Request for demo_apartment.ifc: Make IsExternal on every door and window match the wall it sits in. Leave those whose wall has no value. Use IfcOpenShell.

First a look at what the model holds.

```python
import ifcopenshell
import ifcopenshell.util.element

model = ifcopenshell.open("demo_apartment.ifc")
print(model.schema)
seen = {}
for e in model.by_type("IfcDoor") + model.by_type("IfcWindow"):
    if not e.FillsVoids:
        continue
    host = e.FillsVoids[0].RelatingOpeningElement.VoidsElements[0].RelatingBuildingElement
    own = ifcopenshell.util.element.get_pset(e, f"Pset_{e.is_a()[3:].removesuffix('StandardCase')}Common", "IsExternal")
    wall = ifcopenshell.util.element.get_pset(host, "Pset_WallCommon", "IsExternal")
    seen[e.is_a(), own, wall] = seen.get((e.is_a(), own, wall), 0) + 1
for (cls, own, wall), count in sorted(seen.items(), key=str):
    print(count, cls, "IsExternal:", own, "| host wall:", wall)
```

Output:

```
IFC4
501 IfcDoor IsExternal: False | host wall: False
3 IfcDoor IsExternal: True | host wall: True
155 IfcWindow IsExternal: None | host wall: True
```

```python
import ifcopenshell
import ifcopenshell.api.pset
import ifcopenshell.util.element

model = ifcopenshell.open("demo_apartment.ifc")

count = 0
for ifc_class, pset_name in (("IfcDoor", "Pset_DoorCommon"), ("IfcWindow", "Pset_WindowCommon")):
    for e in model.by_type(ifc_class):
        if not e.FillsVoids:
            continue
        host = e.FillsVoids[0].RelatingOpeningElement.VoidsElements[0].RelatingBuildingElement
        external = ifcopenshell.util.element.get_pset(host, "Pset_WallCommon", "IsExternal")
        if external is None or ifcopenshell.util.element.get_pset(e, pset_name, "IsExternal") == external:
            continue
        pset = ifcopenshell.api.pset.add_pset(model, product=e, name=pset_name)
        ifcopenshell.api.pset.edit_pset(model, pset=pset, properties={"IsExternal": external})
        count += 1

print(count, "updated")

model.write("demo_apartment-out.ifc")
```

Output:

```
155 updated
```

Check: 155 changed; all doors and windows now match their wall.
